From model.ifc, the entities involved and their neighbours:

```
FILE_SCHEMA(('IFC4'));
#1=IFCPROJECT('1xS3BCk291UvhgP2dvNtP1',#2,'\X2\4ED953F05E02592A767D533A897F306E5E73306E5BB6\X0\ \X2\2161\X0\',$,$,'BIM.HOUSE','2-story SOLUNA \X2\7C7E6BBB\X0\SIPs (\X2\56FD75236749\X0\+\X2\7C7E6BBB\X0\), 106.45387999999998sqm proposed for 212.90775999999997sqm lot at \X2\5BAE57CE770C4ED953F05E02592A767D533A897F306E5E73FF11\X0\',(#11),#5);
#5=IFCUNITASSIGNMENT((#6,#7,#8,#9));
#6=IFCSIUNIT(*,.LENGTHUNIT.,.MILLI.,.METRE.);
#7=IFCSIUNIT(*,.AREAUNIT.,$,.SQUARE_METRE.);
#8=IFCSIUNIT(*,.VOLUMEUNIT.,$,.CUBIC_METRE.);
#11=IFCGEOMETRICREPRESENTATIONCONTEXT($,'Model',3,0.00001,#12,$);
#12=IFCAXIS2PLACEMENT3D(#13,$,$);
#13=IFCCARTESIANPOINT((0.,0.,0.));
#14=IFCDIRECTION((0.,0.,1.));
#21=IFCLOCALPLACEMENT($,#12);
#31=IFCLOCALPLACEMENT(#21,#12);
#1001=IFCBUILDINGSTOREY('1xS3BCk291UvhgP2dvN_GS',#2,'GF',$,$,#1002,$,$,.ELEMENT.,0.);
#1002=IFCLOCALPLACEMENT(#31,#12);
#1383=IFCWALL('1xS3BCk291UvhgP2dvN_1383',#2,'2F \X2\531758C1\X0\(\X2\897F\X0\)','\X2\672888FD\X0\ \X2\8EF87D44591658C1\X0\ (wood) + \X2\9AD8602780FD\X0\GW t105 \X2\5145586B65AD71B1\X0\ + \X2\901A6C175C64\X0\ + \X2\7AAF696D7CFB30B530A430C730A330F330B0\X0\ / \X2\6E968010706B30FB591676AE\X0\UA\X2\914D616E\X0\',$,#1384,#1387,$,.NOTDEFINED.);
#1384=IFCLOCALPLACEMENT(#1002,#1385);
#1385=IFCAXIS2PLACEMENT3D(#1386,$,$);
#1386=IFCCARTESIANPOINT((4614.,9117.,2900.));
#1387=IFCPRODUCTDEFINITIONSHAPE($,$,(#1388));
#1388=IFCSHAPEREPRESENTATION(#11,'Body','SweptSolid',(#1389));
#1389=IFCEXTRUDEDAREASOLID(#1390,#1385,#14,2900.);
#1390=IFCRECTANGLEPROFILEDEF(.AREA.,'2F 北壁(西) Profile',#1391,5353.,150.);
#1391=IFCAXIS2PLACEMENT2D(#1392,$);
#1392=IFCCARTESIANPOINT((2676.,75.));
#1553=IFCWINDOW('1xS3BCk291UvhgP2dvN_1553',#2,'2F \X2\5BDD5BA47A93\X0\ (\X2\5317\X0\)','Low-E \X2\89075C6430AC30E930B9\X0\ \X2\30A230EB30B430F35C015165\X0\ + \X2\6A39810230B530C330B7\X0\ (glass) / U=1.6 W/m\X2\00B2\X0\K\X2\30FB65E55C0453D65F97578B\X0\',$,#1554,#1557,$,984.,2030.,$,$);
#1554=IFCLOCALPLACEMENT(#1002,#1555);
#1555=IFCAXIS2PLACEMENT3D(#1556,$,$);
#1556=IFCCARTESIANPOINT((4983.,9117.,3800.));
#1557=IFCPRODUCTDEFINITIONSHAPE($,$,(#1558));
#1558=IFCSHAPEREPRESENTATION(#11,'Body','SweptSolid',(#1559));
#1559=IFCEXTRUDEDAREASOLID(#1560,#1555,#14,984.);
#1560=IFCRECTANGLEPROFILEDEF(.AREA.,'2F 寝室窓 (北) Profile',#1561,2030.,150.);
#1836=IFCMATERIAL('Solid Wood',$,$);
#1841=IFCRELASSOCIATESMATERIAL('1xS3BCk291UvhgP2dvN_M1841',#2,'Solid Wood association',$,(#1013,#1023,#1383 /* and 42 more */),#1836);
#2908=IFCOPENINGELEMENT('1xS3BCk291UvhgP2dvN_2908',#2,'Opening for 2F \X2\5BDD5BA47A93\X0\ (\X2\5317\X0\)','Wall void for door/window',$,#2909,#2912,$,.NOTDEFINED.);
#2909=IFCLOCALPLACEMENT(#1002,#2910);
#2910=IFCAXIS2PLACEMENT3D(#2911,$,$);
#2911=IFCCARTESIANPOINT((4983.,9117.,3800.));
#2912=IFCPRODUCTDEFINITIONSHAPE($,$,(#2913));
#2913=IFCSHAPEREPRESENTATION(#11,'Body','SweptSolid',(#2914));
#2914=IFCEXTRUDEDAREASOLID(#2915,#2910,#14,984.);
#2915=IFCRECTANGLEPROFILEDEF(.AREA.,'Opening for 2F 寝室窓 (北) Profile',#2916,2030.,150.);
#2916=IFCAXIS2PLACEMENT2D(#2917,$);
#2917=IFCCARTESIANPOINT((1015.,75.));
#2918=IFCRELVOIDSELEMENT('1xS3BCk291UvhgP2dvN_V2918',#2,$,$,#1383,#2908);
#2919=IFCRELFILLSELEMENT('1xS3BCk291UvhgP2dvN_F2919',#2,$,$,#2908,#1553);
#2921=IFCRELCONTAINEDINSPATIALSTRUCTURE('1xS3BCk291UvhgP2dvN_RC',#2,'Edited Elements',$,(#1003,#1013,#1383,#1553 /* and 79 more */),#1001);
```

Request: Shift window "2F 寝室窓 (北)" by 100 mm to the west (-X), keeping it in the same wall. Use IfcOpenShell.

```python
import ifcopenshell
import ifcopenshell.api.geometry
import ifcopenshell.util.placement
import ifcopenshell.util.unit

model = ifcopenshell.open("model.ifc")
unit_scale = ifcopenshell.util.unit.calculate_unit_scale(model)

window = model.by_guid("1xS3BCk291UvhgP2dvN_1553")
opening = window.FillsVoids[0].RelatingOpeningElement
wall = opening.VoidsElements[0].RelatingBuildingElement

wall_matrix = ifcopenshell.util.placement.get_local_placement(wall.ObjectPlacement)
shift = wall_matrix[:3, 0] * -0.1 / unit_scale
before = ifcopenshell.util.placement.get_local_placement(window.ObjectPlacement)[:3, 3].copy()

# The window is not placed relative to its opening, so move both.
for product in (opening, window):
    matrix = ifcopenshell.util.placement.get_local_placement(product.ObjectPlacement)
    matrix[:3, 3] += shift
    ifcopenshell.api.geometry.edit_object_placement(model, product=product, matrix=matrix, is_si=False)

after = ifcopenshell.util.placement.get_local_placement(window.ObjectPlacement)[:3, 3]
print("window moved by", (after - before).round(3) + 0.0)

model.write("model_rev.ifc")
```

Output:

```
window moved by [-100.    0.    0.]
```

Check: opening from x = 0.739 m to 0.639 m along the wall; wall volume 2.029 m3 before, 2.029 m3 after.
